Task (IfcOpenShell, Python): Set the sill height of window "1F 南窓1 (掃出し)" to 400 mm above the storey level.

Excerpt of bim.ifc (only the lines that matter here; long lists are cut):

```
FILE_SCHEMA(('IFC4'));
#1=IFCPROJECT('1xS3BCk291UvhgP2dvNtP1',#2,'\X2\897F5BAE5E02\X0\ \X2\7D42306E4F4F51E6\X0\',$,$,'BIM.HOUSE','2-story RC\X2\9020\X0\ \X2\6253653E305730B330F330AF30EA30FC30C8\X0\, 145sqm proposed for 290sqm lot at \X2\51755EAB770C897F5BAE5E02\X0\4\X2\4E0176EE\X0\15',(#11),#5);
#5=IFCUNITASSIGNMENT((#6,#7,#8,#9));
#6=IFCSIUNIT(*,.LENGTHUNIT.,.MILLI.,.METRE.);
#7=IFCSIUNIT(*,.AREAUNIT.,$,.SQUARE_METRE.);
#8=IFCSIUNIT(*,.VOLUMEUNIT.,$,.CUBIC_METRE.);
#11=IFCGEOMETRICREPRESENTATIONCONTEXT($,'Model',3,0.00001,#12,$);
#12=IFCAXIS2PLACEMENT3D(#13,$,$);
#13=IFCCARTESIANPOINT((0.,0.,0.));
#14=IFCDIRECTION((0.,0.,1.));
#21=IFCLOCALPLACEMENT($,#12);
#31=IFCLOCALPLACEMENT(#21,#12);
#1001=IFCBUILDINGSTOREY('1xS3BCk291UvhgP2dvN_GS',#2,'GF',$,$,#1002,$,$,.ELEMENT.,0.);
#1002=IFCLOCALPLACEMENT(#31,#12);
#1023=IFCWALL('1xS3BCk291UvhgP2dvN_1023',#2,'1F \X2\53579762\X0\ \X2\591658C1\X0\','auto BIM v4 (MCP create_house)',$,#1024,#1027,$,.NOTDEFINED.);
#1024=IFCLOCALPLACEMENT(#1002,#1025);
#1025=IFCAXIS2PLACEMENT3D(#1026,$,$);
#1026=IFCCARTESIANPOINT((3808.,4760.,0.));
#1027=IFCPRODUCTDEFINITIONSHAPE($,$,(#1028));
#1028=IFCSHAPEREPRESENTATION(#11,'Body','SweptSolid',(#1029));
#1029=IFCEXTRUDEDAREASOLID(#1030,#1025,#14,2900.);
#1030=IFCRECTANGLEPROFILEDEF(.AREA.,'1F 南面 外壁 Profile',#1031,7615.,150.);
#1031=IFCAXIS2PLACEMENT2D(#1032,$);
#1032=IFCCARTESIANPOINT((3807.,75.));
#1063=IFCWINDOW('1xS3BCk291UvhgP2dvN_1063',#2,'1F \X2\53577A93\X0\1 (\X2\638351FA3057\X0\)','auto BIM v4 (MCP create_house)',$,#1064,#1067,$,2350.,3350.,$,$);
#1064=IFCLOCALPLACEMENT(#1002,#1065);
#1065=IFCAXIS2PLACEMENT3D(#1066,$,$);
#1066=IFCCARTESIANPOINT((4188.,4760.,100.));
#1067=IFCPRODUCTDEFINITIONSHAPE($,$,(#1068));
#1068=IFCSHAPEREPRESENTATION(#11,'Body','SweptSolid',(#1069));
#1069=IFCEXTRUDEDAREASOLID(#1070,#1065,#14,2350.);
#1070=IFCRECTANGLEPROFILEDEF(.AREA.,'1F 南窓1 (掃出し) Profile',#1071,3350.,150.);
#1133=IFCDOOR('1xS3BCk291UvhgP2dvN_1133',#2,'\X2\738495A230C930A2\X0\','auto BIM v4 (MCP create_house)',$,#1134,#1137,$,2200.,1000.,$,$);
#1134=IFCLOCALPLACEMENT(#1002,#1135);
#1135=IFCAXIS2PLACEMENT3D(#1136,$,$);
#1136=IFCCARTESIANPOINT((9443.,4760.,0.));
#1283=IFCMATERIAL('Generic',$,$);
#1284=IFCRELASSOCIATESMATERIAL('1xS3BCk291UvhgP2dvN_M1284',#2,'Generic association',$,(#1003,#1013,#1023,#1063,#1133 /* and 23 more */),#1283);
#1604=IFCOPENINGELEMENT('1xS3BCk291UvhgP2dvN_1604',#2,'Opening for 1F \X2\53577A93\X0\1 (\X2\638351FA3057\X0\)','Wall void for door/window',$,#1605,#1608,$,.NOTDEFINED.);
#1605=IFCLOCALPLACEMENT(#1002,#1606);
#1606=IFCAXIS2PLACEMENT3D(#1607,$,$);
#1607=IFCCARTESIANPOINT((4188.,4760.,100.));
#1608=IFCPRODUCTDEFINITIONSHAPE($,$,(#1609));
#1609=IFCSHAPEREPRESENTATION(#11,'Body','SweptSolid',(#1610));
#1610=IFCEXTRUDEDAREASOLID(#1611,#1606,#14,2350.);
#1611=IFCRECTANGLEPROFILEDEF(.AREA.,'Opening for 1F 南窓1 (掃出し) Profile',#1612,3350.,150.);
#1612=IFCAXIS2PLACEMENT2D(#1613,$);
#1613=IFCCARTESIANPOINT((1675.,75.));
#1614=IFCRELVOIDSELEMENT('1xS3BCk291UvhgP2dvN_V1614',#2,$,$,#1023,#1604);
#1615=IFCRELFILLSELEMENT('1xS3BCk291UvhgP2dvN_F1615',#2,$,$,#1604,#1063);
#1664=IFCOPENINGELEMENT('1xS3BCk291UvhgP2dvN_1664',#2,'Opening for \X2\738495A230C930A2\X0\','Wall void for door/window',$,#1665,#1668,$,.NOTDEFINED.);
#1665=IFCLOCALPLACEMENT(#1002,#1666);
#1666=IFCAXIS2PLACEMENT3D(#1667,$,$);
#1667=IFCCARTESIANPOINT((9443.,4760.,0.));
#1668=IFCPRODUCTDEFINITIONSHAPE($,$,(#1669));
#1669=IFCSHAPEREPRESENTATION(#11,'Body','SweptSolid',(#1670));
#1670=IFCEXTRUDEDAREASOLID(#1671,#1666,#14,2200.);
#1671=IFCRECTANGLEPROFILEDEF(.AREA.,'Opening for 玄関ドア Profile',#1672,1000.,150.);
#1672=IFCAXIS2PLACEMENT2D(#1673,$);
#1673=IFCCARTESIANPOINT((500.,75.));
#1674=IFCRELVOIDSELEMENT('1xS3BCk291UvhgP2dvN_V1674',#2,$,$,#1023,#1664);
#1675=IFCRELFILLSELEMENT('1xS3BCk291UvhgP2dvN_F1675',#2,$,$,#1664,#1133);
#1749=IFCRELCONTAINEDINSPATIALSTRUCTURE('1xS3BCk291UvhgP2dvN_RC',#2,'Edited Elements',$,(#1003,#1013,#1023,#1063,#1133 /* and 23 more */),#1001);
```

```python
import numpy as np
import ifcopenshell
import ifcopenshell.api.geometry
import ifcopenshell.geom
import ifcopenshell.util.element
import ifcopenshell.util.placement
import ifcopenshell.util.shape
import ifcopenshell.util.unit

model = ifcopenshell.open("bim.ifc")
unit_scale = ifcopenshell.util.unit.calculate_unit_scale(model)

window = model.by_id(1063)
opening = window.FillsVoids[0].RelatingOpeningElement
storey = ifcopenshell.util.element.get_container(window, ifc_class="IfcBuildingStorey")
level = ifcopenshell.util.placement.get_local_placement(storey.ObjectPlacement)[2, 3]

# The opening's origin need not be at the sill, so measure its lowest point.
shape = ifcopenshell.geom.create_shape(ifcopenshell.geom.settings(), opening)
bottom = ifcopenshell.util.shape.get_shape_bottom_elevation(shape, shape.geometry) / unit_scale
dz = level + 0.4 / unit_scale - bottom

shift = np.array([0.0, 0.0, dz])
# The window is not placed relative to its opening, so move both.
for product in (opening, window):
    matrix = ifcopenshell.util.placement.get_local_placement(product.ObjectPlacement)
    matrix[:3, 3] += shift
    ifcopenshell.api.geometry.edit_object_placement(model, product=product, matrix=matrix, is_si=False)

print(f"moved by {dz * unit_scale:+.3f} m")

model.write("bim_rev.ifc")
```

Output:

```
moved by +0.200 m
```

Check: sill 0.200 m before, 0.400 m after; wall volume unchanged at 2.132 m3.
